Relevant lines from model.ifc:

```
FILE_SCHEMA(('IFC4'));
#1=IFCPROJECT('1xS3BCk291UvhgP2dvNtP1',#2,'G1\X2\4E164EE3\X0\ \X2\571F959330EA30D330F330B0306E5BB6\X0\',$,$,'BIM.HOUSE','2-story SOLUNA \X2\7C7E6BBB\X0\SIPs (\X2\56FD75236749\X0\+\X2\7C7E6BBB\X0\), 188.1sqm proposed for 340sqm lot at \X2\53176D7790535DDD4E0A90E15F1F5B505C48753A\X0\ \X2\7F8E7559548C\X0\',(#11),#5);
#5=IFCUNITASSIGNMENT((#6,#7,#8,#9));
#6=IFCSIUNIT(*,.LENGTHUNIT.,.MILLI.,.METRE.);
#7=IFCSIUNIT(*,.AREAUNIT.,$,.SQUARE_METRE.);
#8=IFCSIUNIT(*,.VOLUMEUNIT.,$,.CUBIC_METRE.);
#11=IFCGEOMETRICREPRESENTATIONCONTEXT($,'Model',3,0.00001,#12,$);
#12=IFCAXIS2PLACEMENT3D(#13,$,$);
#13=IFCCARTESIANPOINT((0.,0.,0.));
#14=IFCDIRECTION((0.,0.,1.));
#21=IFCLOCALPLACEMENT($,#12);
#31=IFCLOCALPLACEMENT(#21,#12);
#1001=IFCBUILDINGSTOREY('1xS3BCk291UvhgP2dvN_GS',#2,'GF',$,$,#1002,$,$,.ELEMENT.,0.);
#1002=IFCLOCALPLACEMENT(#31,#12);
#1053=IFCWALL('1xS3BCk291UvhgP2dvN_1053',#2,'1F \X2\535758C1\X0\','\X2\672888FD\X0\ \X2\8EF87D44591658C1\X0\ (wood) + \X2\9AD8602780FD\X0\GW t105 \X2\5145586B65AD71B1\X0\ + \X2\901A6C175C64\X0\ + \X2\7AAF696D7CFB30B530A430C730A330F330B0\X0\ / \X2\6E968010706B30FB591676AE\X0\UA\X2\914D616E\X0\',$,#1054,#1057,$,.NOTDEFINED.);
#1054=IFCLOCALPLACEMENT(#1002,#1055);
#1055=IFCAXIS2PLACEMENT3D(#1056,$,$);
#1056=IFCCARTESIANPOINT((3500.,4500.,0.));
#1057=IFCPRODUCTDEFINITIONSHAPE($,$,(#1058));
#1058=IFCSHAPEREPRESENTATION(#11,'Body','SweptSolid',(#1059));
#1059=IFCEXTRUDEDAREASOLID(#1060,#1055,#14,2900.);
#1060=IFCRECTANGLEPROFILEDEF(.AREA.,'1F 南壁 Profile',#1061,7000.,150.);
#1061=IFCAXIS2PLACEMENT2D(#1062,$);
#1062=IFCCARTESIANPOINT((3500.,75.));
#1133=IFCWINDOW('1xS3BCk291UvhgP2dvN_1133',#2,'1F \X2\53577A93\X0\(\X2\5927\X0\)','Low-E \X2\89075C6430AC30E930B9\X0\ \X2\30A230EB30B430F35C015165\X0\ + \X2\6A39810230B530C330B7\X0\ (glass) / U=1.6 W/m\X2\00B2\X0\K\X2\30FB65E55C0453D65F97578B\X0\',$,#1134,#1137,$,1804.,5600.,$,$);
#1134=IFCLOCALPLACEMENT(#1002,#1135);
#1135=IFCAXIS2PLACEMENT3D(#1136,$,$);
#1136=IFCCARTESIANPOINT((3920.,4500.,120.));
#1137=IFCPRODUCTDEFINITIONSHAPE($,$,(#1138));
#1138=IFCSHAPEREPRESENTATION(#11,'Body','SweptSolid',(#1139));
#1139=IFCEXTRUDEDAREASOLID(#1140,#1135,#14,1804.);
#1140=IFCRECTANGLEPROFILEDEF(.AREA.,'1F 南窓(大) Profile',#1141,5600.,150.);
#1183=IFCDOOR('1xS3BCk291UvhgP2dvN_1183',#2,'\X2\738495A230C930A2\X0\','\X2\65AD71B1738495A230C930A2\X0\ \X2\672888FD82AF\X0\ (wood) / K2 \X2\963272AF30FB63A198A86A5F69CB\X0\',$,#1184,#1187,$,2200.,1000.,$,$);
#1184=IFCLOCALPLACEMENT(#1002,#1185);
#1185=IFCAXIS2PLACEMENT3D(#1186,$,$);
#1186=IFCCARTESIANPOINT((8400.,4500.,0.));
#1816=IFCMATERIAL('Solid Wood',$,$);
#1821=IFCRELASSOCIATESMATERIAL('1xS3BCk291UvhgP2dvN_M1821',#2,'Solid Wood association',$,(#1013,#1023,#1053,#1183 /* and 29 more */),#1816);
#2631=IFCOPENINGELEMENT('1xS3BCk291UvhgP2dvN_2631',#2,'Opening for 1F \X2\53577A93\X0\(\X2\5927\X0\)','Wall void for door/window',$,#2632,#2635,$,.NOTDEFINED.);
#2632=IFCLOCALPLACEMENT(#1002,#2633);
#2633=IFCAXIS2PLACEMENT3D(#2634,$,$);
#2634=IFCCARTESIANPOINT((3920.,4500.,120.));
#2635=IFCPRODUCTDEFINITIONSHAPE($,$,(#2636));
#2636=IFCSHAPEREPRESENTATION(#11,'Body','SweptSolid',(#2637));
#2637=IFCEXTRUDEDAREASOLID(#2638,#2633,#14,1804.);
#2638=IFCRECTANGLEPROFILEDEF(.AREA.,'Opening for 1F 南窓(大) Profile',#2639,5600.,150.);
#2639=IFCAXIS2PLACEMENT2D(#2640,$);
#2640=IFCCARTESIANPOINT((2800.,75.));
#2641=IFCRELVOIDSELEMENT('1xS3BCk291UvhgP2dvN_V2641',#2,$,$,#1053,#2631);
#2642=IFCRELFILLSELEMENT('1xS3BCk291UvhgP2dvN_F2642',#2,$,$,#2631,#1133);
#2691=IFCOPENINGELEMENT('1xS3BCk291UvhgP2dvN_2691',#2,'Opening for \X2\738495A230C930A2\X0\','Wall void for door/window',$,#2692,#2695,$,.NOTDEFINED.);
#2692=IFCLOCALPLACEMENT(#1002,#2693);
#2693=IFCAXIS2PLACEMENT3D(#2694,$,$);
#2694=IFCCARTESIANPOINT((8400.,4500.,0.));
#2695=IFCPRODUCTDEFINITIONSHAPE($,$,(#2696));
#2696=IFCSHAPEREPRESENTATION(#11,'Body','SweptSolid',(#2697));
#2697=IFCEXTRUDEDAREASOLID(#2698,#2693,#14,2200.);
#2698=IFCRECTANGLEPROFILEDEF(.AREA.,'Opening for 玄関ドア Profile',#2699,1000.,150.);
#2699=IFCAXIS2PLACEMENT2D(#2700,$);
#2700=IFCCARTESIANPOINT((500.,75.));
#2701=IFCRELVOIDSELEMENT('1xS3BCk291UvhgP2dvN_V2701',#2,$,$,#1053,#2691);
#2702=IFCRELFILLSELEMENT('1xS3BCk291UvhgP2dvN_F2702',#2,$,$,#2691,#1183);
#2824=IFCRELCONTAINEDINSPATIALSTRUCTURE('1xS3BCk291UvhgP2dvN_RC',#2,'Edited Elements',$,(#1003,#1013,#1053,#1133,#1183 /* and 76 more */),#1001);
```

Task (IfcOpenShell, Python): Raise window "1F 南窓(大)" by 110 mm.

```python
import numpy as np
import ifcopenshell
import ifcopenshell.api.geometry
import ifcopenshell.util.placement
import ifcopenshell.util.unit

model = ifcopenshell.open("model.ifc")
unit_scale = ifcopenshell.util.unit.calculate_unit_scale(model)

window = model.by_id(1133)
opening = window.FillsVoids[0].RelatingOpeningElement
dz = 0.11 / unit_scale

shift = np.array([0.0, 0.0, dz])
# The window is not placed relative to its opening, so move both.
for product in (opening, window):
    matrix = ifcopenshell.util.placement.get_local_placement(product.ObjectPlacement)
    matrix[:3, 3] += shift
    ifcopenshell.api.geometry.edit_object_placement(model, product=product, matrix=matrix, is_si=False)

print(f"moved by {dz * unit_scale:+.3f} m")

model.write("model_updated.ifc")
```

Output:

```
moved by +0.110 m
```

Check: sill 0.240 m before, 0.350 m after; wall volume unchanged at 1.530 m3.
